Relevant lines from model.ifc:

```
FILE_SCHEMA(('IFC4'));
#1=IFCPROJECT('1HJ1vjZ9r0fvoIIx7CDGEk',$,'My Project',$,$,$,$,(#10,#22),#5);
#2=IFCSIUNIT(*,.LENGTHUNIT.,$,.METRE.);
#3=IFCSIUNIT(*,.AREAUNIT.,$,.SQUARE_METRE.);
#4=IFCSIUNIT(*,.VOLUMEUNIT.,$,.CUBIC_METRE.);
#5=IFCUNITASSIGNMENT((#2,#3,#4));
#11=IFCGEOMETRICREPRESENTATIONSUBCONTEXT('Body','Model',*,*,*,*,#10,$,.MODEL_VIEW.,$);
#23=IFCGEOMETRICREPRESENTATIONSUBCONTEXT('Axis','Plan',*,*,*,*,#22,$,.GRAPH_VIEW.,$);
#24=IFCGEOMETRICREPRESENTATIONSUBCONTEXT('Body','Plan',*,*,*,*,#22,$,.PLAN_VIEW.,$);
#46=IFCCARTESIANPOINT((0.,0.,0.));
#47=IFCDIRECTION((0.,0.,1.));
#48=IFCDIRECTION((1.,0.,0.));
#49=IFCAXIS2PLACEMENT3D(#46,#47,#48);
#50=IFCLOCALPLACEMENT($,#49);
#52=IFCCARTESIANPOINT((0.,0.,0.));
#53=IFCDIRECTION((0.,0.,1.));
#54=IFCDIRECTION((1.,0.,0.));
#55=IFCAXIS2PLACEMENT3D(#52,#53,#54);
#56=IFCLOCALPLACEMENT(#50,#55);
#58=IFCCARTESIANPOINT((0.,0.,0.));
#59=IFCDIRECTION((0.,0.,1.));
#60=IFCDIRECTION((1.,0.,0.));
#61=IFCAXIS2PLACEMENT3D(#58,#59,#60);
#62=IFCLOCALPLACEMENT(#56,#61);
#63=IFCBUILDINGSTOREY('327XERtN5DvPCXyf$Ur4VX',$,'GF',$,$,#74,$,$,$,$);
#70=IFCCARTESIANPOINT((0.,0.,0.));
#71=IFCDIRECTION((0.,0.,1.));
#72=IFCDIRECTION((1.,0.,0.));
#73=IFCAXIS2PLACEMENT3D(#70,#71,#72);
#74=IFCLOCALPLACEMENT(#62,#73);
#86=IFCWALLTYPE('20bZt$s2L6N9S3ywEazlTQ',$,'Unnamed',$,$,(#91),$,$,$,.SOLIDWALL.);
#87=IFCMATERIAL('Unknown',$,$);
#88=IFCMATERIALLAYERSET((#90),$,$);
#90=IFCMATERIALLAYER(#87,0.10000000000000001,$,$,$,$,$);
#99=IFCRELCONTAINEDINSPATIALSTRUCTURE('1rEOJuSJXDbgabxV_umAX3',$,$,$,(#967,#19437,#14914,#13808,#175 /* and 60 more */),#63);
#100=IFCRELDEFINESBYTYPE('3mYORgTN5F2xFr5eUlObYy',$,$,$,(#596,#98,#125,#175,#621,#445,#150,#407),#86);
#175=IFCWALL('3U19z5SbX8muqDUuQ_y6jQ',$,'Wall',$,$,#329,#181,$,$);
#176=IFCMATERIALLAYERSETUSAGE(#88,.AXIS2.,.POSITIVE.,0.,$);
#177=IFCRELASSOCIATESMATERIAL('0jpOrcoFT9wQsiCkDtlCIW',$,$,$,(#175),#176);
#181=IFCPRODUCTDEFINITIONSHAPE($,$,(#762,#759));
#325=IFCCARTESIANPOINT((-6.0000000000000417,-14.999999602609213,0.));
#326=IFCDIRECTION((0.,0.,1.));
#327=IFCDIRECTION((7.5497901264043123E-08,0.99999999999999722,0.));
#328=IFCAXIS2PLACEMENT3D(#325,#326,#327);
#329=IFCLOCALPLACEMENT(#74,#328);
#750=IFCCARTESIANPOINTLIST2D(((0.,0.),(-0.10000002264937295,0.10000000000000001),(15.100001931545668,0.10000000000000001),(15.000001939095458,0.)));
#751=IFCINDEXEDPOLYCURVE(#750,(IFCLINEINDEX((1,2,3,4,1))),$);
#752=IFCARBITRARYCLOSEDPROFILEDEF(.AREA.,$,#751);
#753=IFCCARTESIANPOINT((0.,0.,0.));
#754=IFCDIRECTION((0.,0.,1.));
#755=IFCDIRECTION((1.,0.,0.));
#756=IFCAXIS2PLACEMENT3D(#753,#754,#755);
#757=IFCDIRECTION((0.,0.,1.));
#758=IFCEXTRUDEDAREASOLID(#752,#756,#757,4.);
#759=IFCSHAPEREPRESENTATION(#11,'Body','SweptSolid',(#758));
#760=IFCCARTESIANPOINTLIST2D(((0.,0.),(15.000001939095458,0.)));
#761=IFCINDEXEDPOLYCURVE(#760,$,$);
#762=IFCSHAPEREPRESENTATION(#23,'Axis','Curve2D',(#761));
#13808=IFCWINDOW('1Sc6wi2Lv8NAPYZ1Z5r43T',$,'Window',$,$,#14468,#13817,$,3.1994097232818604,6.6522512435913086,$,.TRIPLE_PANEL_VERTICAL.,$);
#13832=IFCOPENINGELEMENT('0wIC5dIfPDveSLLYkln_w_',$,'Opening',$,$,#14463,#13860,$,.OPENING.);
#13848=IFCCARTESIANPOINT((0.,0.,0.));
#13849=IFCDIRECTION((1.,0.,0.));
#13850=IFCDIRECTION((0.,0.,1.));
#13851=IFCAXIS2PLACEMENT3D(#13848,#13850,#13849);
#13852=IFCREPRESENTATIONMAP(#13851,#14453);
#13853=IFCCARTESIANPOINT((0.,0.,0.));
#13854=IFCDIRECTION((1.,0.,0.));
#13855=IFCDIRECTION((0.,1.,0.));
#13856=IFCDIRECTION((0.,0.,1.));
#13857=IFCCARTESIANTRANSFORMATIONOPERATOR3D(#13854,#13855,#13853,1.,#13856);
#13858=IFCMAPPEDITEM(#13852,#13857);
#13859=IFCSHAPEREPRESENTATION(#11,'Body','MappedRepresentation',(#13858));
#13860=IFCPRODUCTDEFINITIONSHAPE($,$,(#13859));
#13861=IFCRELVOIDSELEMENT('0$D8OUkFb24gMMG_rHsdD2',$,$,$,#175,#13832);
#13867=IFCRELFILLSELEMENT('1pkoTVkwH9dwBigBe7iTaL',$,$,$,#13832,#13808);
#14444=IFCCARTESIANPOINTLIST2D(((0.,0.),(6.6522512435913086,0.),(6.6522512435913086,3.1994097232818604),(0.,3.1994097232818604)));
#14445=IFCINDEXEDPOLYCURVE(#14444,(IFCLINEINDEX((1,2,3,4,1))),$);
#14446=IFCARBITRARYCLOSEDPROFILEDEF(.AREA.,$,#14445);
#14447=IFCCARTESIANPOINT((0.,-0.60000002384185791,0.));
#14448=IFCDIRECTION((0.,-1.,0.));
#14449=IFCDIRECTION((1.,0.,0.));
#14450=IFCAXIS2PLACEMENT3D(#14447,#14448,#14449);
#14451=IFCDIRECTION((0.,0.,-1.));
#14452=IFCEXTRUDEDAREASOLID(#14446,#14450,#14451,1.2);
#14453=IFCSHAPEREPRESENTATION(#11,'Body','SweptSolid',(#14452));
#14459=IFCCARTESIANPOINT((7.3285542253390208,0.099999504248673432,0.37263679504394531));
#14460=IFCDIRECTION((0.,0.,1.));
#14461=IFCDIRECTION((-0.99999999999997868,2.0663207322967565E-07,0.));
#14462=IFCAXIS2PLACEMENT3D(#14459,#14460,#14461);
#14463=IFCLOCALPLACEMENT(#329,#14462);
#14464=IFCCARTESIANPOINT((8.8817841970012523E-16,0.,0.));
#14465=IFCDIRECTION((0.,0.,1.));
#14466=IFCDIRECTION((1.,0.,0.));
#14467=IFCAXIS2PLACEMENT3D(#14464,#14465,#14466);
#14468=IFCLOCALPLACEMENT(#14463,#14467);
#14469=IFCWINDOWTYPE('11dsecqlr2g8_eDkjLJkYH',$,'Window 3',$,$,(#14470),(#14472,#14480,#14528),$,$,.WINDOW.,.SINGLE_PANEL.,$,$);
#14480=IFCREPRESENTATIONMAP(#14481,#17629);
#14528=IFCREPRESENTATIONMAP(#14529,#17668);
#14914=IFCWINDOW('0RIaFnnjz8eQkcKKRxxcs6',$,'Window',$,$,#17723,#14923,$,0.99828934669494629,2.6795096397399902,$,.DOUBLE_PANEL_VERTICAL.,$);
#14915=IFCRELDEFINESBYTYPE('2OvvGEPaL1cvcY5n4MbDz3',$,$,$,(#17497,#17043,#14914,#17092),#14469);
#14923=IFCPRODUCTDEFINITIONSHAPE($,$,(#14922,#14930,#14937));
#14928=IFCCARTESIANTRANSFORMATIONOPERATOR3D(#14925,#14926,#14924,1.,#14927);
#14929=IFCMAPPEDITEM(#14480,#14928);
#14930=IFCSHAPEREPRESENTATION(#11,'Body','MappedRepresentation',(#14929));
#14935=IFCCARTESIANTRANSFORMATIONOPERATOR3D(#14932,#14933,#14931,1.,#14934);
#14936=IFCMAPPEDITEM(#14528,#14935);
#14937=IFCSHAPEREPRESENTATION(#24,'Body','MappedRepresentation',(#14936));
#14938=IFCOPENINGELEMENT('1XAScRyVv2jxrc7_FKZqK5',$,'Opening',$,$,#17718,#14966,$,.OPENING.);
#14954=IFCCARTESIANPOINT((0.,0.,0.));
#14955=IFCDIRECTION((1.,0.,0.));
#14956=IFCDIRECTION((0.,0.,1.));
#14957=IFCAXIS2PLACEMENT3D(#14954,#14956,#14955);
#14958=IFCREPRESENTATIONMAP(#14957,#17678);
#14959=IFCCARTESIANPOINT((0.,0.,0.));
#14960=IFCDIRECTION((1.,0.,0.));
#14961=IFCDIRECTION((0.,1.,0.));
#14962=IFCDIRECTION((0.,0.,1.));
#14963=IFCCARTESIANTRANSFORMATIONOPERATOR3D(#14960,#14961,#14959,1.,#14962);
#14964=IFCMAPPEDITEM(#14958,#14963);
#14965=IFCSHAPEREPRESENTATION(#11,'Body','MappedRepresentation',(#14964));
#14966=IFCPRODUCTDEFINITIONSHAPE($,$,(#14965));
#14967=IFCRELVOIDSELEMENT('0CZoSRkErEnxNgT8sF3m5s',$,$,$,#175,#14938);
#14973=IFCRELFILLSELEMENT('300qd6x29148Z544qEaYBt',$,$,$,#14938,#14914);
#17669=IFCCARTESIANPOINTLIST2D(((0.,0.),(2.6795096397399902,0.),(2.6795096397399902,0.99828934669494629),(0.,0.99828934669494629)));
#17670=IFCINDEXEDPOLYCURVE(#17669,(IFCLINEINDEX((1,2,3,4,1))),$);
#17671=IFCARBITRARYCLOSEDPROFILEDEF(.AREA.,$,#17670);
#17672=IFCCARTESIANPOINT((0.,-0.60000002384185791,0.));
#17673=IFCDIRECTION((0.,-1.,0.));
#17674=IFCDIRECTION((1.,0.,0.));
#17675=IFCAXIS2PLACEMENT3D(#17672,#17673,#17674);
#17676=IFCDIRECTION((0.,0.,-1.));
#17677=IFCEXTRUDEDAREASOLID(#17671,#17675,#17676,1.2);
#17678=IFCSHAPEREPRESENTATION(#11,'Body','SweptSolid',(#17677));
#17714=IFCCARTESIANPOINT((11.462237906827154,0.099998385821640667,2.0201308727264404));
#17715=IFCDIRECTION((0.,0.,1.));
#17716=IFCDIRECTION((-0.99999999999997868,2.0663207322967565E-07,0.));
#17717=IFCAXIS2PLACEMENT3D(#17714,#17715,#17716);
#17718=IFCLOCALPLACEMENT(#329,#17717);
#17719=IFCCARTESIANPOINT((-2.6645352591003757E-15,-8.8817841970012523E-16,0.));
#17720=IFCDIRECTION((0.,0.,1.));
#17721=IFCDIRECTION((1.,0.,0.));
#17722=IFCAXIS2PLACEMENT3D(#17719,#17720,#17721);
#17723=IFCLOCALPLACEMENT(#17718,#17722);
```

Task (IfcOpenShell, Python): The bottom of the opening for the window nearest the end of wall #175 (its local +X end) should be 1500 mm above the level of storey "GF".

```python
import numpy as np
import ifcopenshell
import ifcopenshell.api.geometry
import ifcopenshell.geom
import ifcopenshell.util.element
import ifcopenshell.util.placement
import ifcopenshell.util.shape
import ifcopenshell.util.unit

model = ifcopenshell.open("model.ifc")
unit_scale = ifcopenshell.util.unit.calculate_unit_scale(model)

window = model.by_guid("0RIaFnnjz8eQkcKKRxxcs6")
opening = window.FillsVoids[0].RelatingOpeningElement
storey = ifcopenshell.util.element.get_container(window, ifc_class="IfcBuildingStorey")
level = ifcopenshell.util.placement.get_local_placement(storey.ObjectPlacement)[2, 3]

# The opening's origin need not be at the sill, so measure its lowest point.
shape = ifcopenshell.geom.create_shape(ifcopenshell.geom.settings(), opening)
bottom = ifcopenshell.util.shape.get_shape_bottom_elevation(shape, shape.geometry) / unit_scale
dz = level + 1.5 / unit_scale - bottom

shift = np.array([0.0, 0.0, dz])
# The window is placed relative to its opening, so it follows when the opening moves.
matrix = ifcopenshell.util.placement.get_local_placement(opening.ObjectPlacement)
matrix[:3, 3] += shift
ifcopenshell.api.geometry.edit_object_placement(
    model, product=opening, matrix=matrix, is_si=False, should_transform_children=True
)

print(f"moved by {dz * unit_scale:+.3f} m")

model.write("model_rev.ifc")
```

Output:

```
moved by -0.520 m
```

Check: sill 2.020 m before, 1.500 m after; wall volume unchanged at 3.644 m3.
